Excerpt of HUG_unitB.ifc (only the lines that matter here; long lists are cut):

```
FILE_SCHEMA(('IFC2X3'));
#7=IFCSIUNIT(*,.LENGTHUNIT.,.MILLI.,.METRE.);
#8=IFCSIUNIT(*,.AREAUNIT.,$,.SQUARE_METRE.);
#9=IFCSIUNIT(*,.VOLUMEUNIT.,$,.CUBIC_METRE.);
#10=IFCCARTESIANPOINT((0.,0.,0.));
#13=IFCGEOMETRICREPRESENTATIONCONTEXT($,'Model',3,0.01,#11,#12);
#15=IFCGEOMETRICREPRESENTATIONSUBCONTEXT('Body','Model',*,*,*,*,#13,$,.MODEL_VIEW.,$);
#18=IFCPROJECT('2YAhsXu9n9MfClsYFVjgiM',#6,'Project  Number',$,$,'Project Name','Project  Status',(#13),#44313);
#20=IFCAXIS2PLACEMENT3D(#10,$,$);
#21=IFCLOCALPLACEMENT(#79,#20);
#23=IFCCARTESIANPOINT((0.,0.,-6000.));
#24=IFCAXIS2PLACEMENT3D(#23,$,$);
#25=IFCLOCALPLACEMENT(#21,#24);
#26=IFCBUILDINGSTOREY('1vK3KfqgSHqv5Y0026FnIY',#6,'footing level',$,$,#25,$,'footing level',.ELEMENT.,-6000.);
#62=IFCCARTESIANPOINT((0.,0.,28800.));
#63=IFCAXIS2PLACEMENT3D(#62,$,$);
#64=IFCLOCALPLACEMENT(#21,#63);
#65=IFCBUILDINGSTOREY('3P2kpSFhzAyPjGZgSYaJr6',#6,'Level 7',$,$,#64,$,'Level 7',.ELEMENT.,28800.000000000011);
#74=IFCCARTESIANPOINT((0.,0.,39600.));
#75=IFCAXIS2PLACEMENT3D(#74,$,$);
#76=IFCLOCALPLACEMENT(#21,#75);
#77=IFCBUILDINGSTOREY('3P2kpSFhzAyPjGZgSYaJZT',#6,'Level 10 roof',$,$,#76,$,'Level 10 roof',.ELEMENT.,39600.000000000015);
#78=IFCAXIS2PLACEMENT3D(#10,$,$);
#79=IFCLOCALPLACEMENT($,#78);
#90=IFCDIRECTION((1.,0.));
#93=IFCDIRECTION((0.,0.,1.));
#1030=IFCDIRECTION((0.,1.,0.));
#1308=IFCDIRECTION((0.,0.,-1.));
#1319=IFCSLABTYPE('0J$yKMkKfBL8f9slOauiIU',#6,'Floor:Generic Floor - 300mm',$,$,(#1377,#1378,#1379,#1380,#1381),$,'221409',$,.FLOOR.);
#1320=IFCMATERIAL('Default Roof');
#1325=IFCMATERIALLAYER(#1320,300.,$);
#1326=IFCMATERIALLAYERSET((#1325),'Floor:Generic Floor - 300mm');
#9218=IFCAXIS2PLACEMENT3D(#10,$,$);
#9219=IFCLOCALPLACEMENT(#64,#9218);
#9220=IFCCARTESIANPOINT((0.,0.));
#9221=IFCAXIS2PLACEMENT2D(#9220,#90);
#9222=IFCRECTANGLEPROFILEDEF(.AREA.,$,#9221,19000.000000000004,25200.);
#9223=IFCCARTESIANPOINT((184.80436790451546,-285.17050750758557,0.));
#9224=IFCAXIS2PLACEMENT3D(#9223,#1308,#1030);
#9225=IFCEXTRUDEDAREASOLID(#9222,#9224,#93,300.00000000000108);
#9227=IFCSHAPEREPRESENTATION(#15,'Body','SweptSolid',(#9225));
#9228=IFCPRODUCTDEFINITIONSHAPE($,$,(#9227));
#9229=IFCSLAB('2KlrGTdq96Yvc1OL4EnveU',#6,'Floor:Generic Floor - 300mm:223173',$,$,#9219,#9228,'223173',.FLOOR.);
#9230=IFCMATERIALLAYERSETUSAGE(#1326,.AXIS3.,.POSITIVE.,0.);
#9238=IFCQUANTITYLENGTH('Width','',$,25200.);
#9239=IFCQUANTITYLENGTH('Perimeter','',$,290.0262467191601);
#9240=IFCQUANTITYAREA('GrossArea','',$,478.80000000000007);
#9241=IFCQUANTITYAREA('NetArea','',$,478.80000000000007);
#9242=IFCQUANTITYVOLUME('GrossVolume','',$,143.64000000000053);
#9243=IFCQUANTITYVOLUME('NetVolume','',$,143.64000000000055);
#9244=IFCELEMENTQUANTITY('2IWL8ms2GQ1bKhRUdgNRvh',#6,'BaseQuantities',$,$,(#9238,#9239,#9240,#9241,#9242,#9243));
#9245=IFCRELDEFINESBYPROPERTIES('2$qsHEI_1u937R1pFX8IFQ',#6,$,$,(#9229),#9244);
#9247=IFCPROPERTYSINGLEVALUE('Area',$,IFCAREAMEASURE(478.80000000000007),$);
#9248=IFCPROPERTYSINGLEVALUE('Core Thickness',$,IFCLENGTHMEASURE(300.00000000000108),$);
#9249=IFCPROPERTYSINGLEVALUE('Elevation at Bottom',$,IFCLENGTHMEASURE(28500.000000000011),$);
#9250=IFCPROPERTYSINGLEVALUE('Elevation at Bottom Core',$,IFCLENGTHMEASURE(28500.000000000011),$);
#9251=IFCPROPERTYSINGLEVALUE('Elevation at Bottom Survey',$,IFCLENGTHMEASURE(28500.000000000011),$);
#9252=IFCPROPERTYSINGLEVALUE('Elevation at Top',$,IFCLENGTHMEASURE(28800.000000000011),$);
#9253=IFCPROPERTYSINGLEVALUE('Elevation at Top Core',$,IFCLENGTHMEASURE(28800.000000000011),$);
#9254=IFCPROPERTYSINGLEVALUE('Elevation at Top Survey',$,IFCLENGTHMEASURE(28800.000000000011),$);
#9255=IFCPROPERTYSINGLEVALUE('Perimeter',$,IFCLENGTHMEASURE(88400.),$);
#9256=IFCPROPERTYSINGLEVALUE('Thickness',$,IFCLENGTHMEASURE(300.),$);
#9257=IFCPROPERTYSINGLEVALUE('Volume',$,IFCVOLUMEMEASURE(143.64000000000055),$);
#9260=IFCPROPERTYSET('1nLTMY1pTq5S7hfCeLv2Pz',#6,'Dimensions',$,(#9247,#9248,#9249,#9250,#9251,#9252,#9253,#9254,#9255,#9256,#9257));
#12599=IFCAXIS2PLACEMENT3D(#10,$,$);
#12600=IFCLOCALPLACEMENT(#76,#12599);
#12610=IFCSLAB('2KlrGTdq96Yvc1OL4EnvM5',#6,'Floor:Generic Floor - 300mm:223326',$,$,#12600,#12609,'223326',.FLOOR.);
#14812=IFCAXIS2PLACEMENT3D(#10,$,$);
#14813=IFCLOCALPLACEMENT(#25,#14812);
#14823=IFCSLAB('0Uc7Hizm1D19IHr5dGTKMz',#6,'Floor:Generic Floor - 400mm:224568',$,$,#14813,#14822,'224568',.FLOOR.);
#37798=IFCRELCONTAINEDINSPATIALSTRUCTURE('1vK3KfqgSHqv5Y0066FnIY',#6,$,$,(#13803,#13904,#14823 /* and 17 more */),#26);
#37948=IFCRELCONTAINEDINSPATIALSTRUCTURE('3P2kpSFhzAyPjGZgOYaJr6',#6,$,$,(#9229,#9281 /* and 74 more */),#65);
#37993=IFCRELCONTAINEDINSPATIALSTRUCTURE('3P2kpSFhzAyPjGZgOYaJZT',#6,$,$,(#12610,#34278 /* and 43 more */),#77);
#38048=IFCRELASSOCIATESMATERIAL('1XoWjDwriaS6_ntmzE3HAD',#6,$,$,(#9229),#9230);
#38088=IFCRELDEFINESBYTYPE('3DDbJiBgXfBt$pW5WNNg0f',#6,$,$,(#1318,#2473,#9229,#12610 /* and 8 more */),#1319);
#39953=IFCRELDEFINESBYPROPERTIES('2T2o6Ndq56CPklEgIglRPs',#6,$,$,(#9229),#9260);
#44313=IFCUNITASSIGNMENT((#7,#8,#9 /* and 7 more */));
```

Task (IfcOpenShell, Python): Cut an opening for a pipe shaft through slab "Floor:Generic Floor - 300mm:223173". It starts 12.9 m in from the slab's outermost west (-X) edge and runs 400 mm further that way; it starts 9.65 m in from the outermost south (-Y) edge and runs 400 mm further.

```python
import numpy as np
import ifcopenshell
import ifcopenshell.api.feature
import ifcopenshell.api.geometry
import ifcopenshell.api.pset
import ifcopenshell.api.root
import ifcopenshell.geom
import ifcopenshell.util.element
import ifcopenshell.util.placement
import ifcopenshell.util.representation
import ifcopenshell.util.shape
import ifcopenshell.util.unit

model = ifcopenshell.open("HUG_unitB.ifc")
unit_scale = ifcopenshell.util.unit.calculate_unit_scale(model)
area_scale = ifcopenshell.util.unit.calculate_unit_scale(model, "AREAUNIT")
volume_scale = ifcopenshell.util.unit.calculate_unit_scale(model, "VOLUMEUNIT")
settings = ifcopenshell.geom.settings()


def volume(element):
    """Net volume in cubic metres, openings subtracted."""
    shape = ifcopenshell.geom.create_shape(settings, element)
    return ifcopenshell.util.shape.get_volume(shape.geometry)


slab = model.by_guid("2KlrGTdq96Yvc1OL4EnveU")
before = volume(slab)

# Extent in the slab's own axes, in metres. The edges named are its -X and -Y sides.
slab_shape = ifcopenshell.geom.create_shape(settings, slab)
vertices = ifcopenshell.util.shape.get_vertices(slab_shape.geometry)
x_min, y_min, bottom = vertices.min(axis=0)
top = vertices[:, 2].max()

opening = ifcopenshell.api.root.create_entity(model, ifc_class="IfcOpeningElement", name="Pipe shaft opening")
context = ifcopenshell.util.representation.get_context(model, "Model", "Body", "MODEL_VIEW")
width, depth = 0.4, 0.4
outline = [(0.0, 0.0), (width, 0.0), (width, depth), (0.0, depth), (0.0, 0.0)]
# Overshoot both faces by 50 mm so the cut is clean.
shape = ifcopenshell.api.geometry.add_slab_representation(
    model, context=context, depth=top - bottom + 0.1, polyline=outline
)
ifcopenshell.api.geometry.assign_representation(model, product=opening, representation=shape)

matrix = ifcopenshell.util.placement.get_local_placement(slab.ObjectPlacement)
matrix[:, 3] = matrix @ np.append(np.array([x_min + 12.9, y_min + 9.65, bottom - 0.05]) / unit_scale, 1.0)
ifcopenshell.api.geometry.edit_object_placement(model, product=opening, matrix=matrix, is_si=False)
ifcopenshell.api.feature.add_feature(model, feature=opening, element=slab)

after = volume(slab)

# Update the slab's stored quantities.
qto = model.by_id(ifcopenshell.util.element.get_pset(slab, "BaseQuantities", should_inherit=False)["id"])
ifcopenshell.api.pset.edit_qto(model, qto=qto, properties={
    "NetArea": after / (top - bottom) / area_scale,
    "NetVolume": after / volume_scale,
})
pset = model.by_id(ifcopenshell.util.element.get_pset(slab, "Dimensions", should_inherit=False)["id"])
ifcopenshell.api.pset.edit_pset(model, pset=pset, properties={
    "Area": model.create_entity("IfcAreaMeasure", after / (top - bottom) / area_scale),
    "Volume": model.create_entity("IfcVolumeMeasure", after / volume_scale),
})

print(f"slab volume {before:.3f} -> {after:.3f} m3")

model.write("HUG_unitB_rev.ifc")
```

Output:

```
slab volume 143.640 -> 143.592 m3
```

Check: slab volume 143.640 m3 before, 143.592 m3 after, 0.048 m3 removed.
